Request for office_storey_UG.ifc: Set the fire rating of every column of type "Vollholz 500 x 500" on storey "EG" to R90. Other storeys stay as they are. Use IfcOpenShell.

First a look at what the model holds.

```python
import ifcopenshell
import ifcopenshell.util.element

model = ifcopenshell.open("office_storey_UG.ifc")
print(model.schema)
storey = next(s for s in model.by_type("IfcBuildingStorey") if s.Name == "EG")
columns = [e for e in ifcopenshell.util.element.get_decomposition(storey) if e.is_a("IfcColumn")]
seen = {}
for e in columns:
    element_type = ifcopenshell.util.element.get_type(e)
    key = (element_type.Name if element_type != e and element_type else None, ifcopenshell.util.element.get_pset(e, "Pset_ColumnCommon", "FireRating"))
    seen[key] = seen.get(key, 0) + 1
for (name, value), count in sorted(seen.items(), key=str):
    print(count, "x", name, "|", value)
```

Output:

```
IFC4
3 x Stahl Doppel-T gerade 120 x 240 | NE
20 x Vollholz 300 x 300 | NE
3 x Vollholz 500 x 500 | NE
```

```python
import ifcopenshell
import ifcopenshell.api.pset
import ifcopenshell.util.element

model = ifcopenshell.open("office_storey_UG.ifc")

storey = next(s for s in model.by_type("IfcBuildingStorey") if s.Name == "EG")
columns = [e for e in ifcopenshell.util.element.get_decomposition(storey) if e.is_a("IfcColumn")]

count = 0
for e in columns:
    element_type = ifcopenshell.util.element.get_type(e)
    if element_type in (None, e) or element_type.Name != "Vollholz 500 x 500":
        continue
    # add_pset returns the element's existing set when there is one.
    pset = ifcopenshell.api.pset.add_pset(model, product=e, name="Pset_ColumnCommon")
    ifcopenshell.api.pset.edit_pset(model, pset=pset, properties={"FireRating": "R90"})
    count += 1

print(count, "columns updated")

model.write("office_storey_UG-out.ifc")
```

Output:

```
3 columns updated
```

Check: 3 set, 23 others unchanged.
